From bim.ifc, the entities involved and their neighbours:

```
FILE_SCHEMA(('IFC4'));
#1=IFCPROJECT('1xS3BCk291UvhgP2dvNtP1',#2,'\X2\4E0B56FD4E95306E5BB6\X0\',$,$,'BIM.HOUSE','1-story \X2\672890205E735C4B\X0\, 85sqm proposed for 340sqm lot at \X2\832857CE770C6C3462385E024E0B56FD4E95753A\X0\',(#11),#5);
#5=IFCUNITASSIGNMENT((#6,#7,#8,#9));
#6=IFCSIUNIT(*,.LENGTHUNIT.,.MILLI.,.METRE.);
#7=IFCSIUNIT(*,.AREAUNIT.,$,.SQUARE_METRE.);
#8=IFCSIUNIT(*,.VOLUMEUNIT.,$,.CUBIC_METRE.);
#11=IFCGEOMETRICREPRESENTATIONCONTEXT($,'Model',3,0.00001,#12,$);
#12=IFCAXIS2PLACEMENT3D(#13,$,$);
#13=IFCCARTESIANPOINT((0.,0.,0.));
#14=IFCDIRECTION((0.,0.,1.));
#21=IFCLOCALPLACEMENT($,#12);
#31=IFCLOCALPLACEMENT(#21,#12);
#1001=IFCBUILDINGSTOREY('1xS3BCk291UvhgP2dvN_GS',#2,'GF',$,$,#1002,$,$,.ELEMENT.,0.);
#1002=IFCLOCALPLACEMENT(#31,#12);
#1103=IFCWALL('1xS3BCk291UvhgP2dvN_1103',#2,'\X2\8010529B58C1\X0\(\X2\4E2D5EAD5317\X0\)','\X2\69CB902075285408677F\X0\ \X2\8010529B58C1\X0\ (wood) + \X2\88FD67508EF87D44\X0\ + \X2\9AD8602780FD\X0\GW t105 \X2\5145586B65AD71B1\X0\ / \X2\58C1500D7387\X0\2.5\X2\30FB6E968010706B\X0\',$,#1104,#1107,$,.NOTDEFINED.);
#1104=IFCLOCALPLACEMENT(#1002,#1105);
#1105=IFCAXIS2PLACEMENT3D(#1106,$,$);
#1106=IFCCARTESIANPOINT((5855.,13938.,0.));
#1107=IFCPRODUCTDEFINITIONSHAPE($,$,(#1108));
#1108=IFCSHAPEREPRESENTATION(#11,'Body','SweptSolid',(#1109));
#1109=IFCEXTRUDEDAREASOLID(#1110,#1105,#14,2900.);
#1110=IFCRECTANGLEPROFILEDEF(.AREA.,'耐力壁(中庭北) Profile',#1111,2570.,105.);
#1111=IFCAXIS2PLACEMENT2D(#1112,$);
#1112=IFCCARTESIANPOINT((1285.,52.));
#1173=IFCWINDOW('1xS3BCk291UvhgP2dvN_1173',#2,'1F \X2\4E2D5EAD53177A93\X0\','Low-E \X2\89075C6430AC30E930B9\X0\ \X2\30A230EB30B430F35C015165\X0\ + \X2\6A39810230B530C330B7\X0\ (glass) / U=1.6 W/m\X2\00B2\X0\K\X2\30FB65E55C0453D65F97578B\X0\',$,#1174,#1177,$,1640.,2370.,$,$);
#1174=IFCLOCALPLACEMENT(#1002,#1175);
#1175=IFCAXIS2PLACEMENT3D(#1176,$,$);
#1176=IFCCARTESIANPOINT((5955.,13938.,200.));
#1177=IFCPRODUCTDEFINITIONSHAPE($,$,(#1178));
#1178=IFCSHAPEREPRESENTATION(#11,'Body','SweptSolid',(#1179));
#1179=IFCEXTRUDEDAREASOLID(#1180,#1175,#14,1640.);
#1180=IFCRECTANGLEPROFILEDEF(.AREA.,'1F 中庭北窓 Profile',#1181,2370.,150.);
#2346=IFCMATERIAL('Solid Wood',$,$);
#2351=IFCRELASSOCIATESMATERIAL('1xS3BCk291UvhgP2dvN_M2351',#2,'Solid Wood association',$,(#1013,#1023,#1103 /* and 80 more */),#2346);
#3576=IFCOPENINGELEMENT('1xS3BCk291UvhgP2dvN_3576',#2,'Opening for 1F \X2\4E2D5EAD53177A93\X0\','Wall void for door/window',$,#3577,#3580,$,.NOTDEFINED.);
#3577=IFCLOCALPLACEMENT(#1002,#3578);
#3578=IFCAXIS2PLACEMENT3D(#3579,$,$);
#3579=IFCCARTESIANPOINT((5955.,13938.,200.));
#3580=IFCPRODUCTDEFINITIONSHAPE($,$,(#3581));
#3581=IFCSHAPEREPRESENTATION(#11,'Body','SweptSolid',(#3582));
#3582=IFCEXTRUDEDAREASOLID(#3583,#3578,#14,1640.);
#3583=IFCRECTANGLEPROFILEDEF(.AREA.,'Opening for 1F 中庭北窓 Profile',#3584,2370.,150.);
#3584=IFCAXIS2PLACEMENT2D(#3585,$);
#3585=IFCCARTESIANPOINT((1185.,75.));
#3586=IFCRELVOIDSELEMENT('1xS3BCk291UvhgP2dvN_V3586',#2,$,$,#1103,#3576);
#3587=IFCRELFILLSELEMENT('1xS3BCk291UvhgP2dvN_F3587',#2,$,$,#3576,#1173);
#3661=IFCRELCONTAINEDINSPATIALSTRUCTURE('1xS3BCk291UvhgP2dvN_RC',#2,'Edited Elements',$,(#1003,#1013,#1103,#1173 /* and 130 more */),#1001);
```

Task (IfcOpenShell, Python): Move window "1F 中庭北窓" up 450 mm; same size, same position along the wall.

```python
import numpy as np
import ifcopenshell
import ifcopenshell.api.geometry
import ifcopenshell.util.placement
import ifcopenshell.util.unit

model = ifcopenshell.open("bim.ifc")
unit_scale = ifcopenshell.util.unit.calculate_unit_scale(model)

window = model.by_guid("1xS3BCk291UvhgP2dvN_1173")
opening = window.FillsVoids[0].RelatingOpeningElement
dz = 450.0

shift = np.array([0.0, 0.0, dz])
# The window is not placed relative to its opening, so move both.
for product in (opening, window):
    matrix = ifcopenshell.util.placement.get_local_placement(product.ObjectPlacement)
    matrix[:3, 3] += shift
    ifcopenshell.api.geometry.edit_object_placement(model, product=product, matrix=matrix, is_si=False)

print(f"moved by {dz * unit_scale:+.3f} m")

model.write("bim_rev.ifc")
```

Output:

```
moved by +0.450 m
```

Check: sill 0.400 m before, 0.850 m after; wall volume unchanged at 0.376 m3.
